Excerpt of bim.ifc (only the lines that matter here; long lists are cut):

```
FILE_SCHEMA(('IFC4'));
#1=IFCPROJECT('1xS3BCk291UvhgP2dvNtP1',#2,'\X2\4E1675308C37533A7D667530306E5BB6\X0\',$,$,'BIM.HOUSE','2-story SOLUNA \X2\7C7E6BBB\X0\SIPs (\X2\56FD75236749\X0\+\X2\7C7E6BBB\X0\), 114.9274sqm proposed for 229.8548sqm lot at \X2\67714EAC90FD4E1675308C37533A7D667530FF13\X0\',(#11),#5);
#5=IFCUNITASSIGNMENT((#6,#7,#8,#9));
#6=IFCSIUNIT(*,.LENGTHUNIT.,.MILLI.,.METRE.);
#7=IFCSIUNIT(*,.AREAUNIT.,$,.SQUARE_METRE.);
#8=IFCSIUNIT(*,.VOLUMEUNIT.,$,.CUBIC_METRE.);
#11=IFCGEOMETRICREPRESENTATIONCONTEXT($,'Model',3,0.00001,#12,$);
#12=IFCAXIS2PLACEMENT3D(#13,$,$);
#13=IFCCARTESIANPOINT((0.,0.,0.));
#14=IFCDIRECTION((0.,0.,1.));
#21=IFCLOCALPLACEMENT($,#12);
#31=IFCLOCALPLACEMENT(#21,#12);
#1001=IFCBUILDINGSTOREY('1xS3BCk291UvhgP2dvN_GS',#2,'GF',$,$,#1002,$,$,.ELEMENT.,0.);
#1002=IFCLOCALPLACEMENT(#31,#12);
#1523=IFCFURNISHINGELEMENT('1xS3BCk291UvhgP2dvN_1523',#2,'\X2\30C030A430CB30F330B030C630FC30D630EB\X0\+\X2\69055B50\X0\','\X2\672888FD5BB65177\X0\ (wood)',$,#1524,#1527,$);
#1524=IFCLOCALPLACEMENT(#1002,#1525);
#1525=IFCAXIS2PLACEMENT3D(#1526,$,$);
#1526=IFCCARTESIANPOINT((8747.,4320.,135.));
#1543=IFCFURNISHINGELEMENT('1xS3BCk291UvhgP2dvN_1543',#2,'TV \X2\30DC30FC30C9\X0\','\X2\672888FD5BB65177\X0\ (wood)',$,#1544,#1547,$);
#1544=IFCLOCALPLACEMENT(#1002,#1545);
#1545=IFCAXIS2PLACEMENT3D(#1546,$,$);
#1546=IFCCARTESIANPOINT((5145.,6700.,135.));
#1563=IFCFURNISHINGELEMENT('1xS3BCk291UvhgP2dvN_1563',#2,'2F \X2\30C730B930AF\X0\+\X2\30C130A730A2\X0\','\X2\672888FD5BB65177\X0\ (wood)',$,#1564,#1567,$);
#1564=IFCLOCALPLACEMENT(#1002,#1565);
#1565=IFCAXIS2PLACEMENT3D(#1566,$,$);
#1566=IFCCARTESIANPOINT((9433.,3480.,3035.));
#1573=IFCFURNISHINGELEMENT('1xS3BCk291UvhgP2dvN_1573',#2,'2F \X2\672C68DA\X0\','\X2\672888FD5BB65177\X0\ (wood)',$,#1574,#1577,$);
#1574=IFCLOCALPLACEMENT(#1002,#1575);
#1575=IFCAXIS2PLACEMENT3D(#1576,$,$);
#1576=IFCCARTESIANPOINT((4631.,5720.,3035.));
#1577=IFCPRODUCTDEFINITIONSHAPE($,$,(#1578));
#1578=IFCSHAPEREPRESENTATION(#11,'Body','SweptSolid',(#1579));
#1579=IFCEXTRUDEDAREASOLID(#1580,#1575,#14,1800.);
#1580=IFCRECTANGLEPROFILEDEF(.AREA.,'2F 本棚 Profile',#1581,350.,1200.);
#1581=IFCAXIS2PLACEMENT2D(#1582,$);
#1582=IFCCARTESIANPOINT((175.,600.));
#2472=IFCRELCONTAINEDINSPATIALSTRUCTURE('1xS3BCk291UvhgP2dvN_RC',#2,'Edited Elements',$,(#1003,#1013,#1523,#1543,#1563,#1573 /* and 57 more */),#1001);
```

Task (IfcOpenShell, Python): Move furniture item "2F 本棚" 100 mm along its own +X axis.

```python
import ifcopenshell
import ifcopenshell.api.geometry
import ifcopenshell.util.placement
import ifcopenshell.util.unit

model = ifcopenshell.open("bim.ifc")
unit_scale = ifcopenshell.util.unit.calculate_unit_scale(model)

item = model.by_guid("1xS3BCk291UvhgP2dvN_1573")
matrix = ifcopenshell.util.placement.get_local_placement(item.ObjectPlacement)
matrix[:3, 3] += matrix[:3, 0] * 0.1 / unit_scale
ifcopenshell.api.geometry.edit_object_placement(model, product=item, matrix=matrix, is_si=False)

print(ifcopenshell.util.placement.get_local_placement(item.ObjectPlacement).round(3) + 0.0)

model.write("bim-out.ifc")
```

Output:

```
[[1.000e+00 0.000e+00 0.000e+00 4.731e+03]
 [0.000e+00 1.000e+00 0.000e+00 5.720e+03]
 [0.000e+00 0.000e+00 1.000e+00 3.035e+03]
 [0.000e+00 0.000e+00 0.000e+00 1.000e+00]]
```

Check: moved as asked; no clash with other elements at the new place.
